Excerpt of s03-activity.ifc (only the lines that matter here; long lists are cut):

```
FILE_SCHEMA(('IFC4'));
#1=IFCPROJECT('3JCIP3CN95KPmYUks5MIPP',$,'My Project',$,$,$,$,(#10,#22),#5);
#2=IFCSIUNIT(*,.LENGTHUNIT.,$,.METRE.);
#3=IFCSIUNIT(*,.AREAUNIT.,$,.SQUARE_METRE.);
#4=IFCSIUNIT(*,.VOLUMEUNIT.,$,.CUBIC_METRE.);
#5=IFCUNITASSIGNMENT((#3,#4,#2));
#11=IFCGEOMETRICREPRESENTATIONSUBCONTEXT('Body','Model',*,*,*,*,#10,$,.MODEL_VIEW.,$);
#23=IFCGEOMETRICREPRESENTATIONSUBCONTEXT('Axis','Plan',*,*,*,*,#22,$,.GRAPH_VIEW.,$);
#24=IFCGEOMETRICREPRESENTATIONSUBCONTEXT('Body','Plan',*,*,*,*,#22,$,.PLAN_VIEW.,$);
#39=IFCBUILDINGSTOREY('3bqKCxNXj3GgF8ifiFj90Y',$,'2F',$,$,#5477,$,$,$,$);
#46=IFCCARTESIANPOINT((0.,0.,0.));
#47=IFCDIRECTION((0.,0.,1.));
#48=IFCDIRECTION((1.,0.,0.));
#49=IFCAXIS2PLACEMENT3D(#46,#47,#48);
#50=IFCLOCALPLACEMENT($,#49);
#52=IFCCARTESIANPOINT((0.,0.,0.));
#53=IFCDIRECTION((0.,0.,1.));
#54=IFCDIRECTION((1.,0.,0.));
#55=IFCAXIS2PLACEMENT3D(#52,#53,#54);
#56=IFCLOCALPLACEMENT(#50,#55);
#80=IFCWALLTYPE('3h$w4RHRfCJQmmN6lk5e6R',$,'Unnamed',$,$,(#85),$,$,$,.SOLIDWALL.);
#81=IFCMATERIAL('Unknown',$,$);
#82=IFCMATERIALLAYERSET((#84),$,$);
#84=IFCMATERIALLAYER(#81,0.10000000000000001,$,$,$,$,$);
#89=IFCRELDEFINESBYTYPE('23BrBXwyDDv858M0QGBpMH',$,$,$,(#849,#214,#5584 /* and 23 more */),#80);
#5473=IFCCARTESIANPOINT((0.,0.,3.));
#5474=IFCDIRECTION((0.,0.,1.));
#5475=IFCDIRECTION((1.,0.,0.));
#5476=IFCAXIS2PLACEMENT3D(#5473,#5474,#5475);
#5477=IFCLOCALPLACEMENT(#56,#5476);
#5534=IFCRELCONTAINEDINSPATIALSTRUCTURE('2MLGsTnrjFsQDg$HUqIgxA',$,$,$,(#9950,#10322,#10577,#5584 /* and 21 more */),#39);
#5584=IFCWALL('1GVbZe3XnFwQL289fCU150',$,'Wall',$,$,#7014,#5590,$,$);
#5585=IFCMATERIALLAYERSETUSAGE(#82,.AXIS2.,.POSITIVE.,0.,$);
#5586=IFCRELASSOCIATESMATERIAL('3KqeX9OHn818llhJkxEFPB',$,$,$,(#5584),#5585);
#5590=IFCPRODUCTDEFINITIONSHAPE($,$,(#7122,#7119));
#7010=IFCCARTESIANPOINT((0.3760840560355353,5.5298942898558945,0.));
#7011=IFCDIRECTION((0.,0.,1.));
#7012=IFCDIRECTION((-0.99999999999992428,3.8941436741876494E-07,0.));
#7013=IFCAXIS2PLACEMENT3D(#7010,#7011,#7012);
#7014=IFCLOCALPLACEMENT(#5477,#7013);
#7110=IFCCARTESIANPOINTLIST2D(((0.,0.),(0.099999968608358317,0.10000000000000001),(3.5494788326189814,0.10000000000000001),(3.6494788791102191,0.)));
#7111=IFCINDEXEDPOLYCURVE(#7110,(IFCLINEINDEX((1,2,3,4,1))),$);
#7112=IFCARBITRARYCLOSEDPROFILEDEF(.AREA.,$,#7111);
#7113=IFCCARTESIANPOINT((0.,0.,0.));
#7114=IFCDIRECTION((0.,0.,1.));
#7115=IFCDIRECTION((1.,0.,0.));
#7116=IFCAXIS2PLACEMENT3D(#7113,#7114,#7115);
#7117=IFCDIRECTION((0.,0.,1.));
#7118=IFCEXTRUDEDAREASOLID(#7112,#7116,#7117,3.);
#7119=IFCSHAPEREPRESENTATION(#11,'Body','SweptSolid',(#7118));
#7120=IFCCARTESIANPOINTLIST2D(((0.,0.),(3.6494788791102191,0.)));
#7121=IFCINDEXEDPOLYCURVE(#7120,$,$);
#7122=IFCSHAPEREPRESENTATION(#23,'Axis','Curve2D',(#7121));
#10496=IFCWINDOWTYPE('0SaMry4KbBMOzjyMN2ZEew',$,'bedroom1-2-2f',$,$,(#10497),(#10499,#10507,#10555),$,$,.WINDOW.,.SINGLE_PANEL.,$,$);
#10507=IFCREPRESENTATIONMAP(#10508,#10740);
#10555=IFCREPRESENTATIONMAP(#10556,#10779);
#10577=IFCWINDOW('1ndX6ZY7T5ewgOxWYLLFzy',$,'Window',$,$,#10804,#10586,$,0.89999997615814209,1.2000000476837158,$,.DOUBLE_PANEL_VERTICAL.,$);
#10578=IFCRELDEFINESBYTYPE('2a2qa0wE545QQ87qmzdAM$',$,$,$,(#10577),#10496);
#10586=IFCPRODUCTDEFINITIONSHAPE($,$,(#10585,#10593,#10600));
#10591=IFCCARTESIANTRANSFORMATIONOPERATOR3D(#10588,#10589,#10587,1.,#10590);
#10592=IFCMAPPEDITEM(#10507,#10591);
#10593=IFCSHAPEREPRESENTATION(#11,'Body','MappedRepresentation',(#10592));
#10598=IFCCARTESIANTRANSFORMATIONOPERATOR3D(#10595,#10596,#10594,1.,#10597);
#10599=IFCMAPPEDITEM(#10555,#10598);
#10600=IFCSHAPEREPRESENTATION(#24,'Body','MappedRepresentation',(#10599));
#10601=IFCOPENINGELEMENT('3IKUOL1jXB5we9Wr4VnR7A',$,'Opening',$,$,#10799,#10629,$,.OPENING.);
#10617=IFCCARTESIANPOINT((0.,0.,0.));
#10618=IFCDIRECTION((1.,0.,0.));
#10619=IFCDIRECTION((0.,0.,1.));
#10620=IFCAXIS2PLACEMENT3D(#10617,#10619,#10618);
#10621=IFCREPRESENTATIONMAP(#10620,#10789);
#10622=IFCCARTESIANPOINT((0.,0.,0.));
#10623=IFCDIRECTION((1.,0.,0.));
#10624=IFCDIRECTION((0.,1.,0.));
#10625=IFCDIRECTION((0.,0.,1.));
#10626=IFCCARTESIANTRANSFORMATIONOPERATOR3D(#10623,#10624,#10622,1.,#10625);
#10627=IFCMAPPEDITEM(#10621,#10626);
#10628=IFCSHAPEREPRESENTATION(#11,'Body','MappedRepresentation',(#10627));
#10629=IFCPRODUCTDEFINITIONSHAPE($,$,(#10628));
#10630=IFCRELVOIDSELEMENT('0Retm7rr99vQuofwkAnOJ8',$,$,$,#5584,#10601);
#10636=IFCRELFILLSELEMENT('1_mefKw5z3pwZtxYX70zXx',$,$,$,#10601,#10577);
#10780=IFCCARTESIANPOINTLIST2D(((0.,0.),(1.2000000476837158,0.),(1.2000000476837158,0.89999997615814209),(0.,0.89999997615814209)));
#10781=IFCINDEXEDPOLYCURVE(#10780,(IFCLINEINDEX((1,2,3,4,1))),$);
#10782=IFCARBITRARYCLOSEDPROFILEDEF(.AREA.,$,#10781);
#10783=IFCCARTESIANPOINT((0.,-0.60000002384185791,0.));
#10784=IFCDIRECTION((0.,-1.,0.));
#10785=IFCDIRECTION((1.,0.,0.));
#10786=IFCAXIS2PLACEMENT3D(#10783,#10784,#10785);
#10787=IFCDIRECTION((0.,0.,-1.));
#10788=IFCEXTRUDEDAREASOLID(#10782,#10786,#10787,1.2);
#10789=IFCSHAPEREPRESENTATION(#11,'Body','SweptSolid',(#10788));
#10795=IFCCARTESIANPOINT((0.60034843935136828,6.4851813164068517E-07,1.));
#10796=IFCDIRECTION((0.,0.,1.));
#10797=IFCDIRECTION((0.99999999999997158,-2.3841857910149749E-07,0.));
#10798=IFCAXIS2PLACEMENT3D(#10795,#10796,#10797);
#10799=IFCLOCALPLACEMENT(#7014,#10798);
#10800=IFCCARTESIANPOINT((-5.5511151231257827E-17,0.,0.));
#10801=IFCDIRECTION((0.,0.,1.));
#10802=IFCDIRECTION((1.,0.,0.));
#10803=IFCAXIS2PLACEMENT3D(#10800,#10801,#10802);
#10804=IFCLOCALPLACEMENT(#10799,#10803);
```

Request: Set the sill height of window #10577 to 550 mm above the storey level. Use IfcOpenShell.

```python
import numpy as np
import ifcopenshell
import ifcopenshell.api.geometry
import ifcopenshell.geom
import ifcopenshell.util.element
import ifcopenshell.util.placement
import ifcopenshell.util.shape
import ifcopenshell.util.unit

model = ifcopenshell.open("s03-activity.ifc")
unit_scale = ifcopenshell.util.unit.calculate_unit_scale(model)

window = model.by_guid("1ndX6ZY7T5ewgOxWYLLFzy")
opening = window.FillsVoids[0].RelatingOpeningElement
storey = ifcopenshell.util.element.get_container(window, ifc_class="IfcBuildingStorey")
level = ifcopenshell.util.placement.get_local_placement(storey.ObjectPlacement)[2, 3]

# The opening's origin need not be at the sill, so measure its lowest point.
shape = ifcopenshell.geom.create_shape(ifcopenshell.geom.settings(), opening)
bottom = ifcopenshell.util.shape.get_shape_bottom_elevation(shape, shape.geometry) / unit_scale
dz = level + 0.55 - bottom

shift = np.array([0.0, 0.0, dz])
# The window is placed relative to its opening, so it follows when the opening moves.
matrix = ifcopenshell.util.placement.get_local_placement(opening.ObjectPlacement)
matrix[:3, 3] += shift
ifcopenshell.api.geometry.edit_object_placement(
    model, product=opening, matrix=matrix, is_si=False, should_transform_children=True
)

print(f"moved by {dz * unit_scale:+.3f} m")

model.write("s03-activity_rev.ifc")
```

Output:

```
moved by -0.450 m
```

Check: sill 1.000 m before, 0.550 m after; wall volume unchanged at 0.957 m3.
